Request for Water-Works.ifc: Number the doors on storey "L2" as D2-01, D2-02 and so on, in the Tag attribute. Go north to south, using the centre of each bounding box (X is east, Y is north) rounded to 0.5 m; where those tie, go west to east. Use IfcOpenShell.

First a look at what the model holds.

```python
import ifcopenshell
import ifcopenshell.util.element
import ifcopenshell.util.placement

model = ifcopenshell.open("Water-Works.ifc")
print(model.schema)
storey = next(s for s in model.by_type("IfcBuildingStorey") if s.Name == "L2")
doors = [e for e in ifcopenshell.util.element.get_decomposition(storey) if e.is_a("IfcDoor")]
for e in sorted(doors, key=lambda e: e.id()):
    origin = ifcopenshell.util.placement.get_local_placement(e.ObjectPlacement)[:3, 3]
    print(e.id(), e.Tag, e.Name, origin.round(2) + 0.0, sep=" | ")
```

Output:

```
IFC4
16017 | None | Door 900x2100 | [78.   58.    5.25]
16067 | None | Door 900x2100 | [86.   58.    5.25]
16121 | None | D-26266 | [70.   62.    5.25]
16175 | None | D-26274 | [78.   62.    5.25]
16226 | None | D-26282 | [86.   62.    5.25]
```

```python
import ifcopenshell
import ifcopenshell.geom
import ifcopenshell.util.element
import ifcopenshell.util.shape

model = ifcopenshell.open("Water-Works.ifc")
settings = ifcopenshell.geom.settings()
settings.set("use-world-coords", True)


def centre(element):
    shape = ifcopenshell.geom.create_shape(settings, element)
    return ifcopenshell.util.shape.get_bbox_centroid(shape.geometry)


storey = next(s for s in model.by_type("IfcBuildingStorey") if s.Name == "L2")
doors = [e for e in ifcopenshell.util.element.get_decomposition(storey) if e.is_a("IfcDoor")]

# Insertion points can sit at a corner or the storey origin, so sort by the geometry (in metres).
centres = {e: centre(e) for e in doors}
doors.sort(key=lambda e: (-round(centres[e][1] / 0.5), centres[e][0]))

for i, e in enumerate(doors, start=1):
    number = f"D2-{i:02d}"
    e.Tag = number
    print(e.id(), number)

model.write("Water-Works_rev.ifc")
```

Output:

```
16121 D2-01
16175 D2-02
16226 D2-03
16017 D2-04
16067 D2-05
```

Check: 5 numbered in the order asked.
